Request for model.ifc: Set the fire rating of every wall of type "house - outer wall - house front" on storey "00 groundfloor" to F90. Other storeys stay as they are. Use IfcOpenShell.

First a look at what the model holds.

```python
import ifcopenshell
import ifcopenshell.util.element

model = ifcopenshell.open("model.ifc")
print(model.schema)
storey = next(s for s in model.by_type("IfcBuildingStorey") if s.Name == "00 groundfloor")
walls = [e for e in ifcopenshell.util.element.get_decomposition(storey) if e.is_a("IfcWall")]
seen = {}
for e in walls:
    element_type = ifcopenshell.util.element.get_type(e)
    key = (element_type.Name if element_type != e and element_type else None, ifcopenshell.util.element.get_pset(e, "Pset_WallCommon", "FireRating"))
    seen[key] = seen.get(key, 0) + 1
for (name, value), count in sorted(seen.items(), key=str):
    print(count, "x", name, "|", value)
```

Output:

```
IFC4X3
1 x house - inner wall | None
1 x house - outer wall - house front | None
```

```python
import ifcopenshell
import ifcopenshell.api.pset
import ifcopenshell.util.element

model = ifcopenshell.open("model.ifc")

storey = next(s for s in model.by_type("IfcBuildingStorey") if s.Name == "00 groundfloor")
walls = [e for e in ifcopenshell.util.element.get_decomposition(storey) if e.is_a("IfcWall")]

count = 0
for e in walls:
    element_type = ifcopenshell.util.element.get_type(e)
    if element_type in (None, e) or element_type.Name != "house - outer wall - house front":
        continue
    # add_pset returns the element's existing set when there is one.
    pset = ifcopenshell.api.pset.add_pset(model, product=e, name="Pset_WallCommon")
    ifcopenshell.api.pset.edit_pset(model, pset=pset, properties={"FireRating": "F90"})
    count += 1

print(count, "walls updated")

model.write("model_v2.ifc")
```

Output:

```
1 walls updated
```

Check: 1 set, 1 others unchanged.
